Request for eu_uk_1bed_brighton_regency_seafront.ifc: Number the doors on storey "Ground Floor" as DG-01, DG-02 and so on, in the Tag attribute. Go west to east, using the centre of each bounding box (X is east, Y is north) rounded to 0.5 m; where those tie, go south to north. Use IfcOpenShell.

First a look at what the model holds.

```python
import ifcopenshell
import ifcopenshell.util.element
import ifcopenshell.util.placement

model = ifcopenshell.open("eu_uk_1bed_brighton_regency_seafront.ifc")
print(model.schema)
storey = next(s for s in model.by_type("IfcBuildingStorey") if s.Name == "Ground Floor")
doors = [e for e in ifcopenshell.util.element.get_decomposition(storey) if e.is_a("IfcDoor")]
for e in sorted(doors, key=lambda e: e.id()):
    origin = ifcopenshell.util.placement.get_local_placement(e.ObjectPlacement)[:3, 3]
    print(e.id(), e.Tag, e.Name, origin.round(2) + 0.0, sep=" | ")
```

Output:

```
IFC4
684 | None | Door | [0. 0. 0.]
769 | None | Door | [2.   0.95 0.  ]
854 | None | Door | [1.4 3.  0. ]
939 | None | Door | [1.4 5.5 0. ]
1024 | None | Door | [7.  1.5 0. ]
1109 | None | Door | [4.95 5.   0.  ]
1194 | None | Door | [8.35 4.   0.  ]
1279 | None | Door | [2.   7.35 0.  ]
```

```python
import ifcopenshell
import ifcopenshell.geom
import ifcopenshell.util.element
import ifcopenshell.util.shape

model = ifcopenshell.open("eu_uk_1bed_brighton_regency_seafront.ifc")
settings = ifcopenshell.geom.settings()
settings.set("use-world-coords", True)


def centre(element):
    shape = ifcopenshell.geom.create_shape(settings, element)
    return ifcopenshell.util.shape.get_bbox_centroid(shape.geometry)


storey = next(s for s in model.by_type("IfcBuildingStorey") if s.Name == "Ground Floor")
doors = [e for e in ifcopenshell.util.element.get_decomposition(storey) if e.is_a("IfcDoor")]

# Insertion points can sit at a corner or the storey origin, so sort by the geometry (in metres).
centres = {e: centre(e) for e in doors}
doors.sort(key=lambda e: (round(centres[e][0] / 0.5), centres[e][1]))

for i, e in enumerate(doors, start=1):
    number = f"DG-{i:02d}"
    e.Tag = number
    print(e.id(), number)

model.write("eu_uk_1bed_brighton_regency_seafront_v2.ifc")
```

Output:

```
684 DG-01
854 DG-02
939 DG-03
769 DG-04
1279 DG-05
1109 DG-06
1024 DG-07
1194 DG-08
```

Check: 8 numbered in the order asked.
